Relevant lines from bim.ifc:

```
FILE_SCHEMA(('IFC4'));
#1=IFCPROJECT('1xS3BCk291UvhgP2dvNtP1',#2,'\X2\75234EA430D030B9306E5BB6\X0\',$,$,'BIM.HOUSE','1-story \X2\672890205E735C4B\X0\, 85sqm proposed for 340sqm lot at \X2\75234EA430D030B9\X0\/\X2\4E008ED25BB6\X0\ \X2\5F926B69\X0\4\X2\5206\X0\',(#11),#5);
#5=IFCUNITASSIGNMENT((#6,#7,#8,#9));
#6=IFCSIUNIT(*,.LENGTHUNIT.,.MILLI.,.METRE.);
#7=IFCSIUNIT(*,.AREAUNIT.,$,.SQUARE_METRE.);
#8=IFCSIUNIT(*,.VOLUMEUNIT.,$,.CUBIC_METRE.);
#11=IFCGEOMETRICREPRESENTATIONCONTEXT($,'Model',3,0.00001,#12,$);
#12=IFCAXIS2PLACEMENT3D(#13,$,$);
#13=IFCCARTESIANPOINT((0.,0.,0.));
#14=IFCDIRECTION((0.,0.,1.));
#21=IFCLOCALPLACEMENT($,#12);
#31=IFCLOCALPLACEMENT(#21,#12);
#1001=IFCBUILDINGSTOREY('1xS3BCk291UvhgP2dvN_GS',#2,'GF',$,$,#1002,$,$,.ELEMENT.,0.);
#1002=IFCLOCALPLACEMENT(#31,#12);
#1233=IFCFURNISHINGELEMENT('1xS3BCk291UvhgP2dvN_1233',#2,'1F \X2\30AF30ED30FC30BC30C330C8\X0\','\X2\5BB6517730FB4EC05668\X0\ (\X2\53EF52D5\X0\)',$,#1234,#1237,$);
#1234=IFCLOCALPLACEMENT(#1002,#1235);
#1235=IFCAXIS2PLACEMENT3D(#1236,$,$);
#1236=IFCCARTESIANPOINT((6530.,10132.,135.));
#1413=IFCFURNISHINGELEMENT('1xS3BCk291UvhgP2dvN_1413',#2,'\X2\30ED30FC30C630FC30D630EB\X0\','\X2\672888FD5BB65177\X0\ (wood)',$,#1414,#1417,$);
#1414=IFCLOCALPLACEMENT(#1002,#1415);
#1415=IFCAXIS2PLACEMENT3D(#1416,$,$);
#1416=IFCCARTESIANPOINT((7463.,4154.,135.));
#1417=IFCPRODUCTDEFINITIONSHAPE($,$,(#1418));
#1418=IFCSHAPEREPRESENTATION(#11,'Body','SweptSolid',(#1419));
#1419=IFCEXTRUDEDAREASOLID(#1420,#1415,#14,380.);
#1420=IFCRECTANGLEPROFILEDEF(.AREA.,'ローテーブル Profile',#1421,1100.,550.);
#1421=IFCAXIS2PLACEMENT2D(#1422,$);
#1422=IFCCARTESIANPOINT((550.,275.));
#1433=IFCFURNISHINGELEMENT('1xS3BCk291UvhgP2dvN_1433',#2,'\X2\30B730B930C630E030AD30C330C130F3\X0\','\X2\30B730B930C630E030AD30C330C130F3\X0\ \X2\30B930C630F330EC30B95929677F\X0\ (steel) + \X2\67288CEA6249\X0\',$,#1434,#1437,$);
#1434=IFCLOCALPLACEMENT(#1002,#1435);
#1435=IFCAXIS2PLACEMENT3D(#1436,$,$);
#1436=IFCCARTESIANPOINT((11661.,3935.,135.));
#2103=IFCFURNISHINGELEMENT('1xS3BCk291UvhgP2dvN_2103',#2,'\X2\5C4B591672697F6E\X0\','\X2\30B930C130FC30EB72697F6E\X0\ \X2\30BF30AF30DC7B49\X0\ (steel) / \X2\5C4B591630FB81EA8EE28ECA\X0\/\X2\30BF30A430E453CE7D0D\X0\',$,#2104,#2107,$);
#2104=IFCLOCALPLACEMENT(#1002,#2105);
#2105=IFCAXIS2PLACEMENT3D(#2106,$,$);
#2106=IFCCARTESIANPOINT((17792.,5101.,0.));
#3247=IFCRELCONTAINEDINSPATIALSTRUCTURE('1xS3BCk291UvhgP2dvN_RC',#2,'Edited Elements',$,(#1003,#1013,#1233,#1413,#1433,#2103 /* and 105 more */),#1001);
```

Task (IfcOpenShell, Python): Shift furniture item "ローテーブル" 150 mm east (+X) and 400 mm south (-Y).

```python
import ifcopenshell
import ifcopenshell.api.geometry
import ifcopenshell.util.placement

model = ifcopenshell.open("bim.ifc")

item = model.by_id(1413)
matrix = ifcopenshell.util.placement.get_local_placement(item.ObjectPlacement)
matrix[0, 3] += 150.0
matrix[1, 3] -= 400.0
ifcopenshell.api.geometry.edit_object_placement(model, product=item, matrix=matrix, is_si=False)

print(ifcopenshell.util.placement.get_local_placement(item.ObjectPlacement).round(3) + 0.0)

model.write("bim_v2.ifc")
```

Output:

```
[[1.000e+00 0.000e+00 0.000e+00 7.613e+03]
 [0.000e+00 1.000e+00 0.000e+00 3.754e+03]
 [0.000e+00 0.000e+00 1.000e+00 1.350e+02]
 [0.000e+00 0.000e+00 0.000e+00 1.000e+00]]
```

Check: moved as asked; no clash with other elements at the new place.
